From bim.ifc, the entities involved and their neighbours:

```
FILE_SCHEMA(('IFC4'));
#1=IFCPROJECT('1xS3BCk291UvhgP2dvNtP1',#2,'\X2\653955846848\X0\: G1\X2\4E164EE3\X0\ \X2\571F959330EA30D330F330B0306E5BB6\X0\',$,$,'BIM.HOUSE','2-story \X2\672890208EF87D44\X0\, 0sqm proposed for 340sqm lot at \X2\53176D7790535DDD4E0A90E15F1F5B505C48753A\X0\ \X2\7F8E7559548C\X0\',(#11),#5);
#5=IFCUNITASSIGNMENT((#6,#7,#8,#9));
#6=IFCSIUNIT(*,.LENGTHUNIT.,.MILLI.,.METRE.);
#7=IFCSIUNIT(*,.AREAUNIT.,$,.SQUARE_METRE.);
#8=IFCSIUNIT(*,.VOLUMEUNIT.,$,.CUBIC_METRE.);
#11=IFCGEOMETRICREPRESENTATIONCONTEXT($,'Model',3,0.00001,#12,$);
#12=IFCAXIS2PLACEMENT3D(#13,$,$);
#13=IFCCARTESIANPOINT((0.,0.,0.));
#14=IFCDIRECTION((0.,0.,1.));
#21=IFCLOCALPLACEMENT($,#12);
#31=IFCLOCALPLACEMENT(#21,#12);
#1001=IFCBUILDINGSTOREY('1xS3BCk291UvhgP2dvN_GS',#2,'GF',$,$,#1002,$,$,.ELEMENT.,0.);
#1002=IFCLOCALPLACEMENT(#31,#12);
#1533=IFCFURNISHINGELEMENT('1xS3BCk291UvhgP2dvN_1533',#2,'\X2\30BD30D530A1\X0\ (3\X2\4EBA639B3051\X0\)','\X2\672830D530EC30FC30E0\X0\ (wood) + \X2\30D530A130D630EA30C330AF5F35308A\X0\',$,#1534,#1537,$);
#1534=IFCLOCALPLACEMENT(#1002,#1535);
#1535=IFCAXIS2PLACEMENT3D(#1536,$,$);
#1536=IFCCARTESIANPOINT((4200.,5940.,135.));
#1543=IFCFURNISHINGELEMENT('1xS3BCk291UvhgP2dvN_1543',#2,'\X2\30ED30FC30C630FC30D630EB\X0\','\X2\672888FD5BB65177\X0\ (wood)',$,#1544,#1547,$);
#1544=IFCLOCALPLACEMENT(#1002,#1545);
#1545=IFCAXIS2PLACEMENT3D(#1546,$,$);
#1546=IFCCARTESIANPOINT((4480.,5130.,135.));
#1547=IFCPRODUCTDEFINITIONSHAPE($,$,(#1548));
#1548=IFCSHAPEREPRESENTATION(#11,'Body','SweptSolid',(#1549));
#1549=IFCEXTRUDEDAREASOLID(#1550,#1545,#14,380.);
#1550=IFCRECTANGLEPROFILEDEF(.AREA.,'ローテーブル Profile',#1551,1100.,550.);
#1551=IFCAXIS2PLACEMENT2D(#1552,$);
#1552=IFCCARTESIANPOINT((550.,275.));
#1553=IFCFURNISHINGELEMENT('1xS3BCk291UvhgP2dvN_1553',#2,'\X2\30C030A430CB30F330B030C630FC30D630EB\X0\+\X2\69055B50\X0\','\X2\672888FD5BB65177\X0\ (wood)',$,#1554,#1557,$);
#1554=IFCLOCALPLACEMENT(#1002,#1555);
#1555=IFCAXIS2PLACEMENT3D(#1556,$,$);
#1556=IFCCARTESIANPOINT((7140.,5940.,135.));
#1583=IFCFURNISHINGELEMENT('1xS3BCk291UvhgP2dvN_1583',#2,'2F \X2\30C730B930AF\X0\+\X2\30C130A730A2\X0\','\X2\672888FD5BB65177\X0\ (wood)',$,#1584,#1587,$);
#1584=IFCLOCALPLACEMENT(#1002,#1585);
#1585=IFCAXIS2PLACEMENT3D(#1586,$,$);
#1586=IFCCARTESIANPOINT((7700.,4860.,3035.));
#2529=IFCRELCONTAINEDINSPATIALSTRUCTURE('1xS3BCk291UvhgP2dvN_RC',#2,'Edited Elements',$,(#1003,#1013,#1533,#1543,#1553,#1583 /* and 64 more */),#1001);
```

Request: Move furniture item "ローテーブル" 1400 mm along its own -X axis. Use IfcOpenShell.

```python
import ifcopenshell
import ifcopenshell.api.geometry
import ifcopenshell.util.placement

model = ifcopenshell.open("bim.ifc")

item = model.by_guid("1xS3BCk291UvhgP2dvN_1543")
matrix = ifcopenshell.util.placement.get_local_placement(item.ObjectPlacement)
matrix[:3, 3] -= matrix[:3, 0] * 1400.0
ifcopenshell.api.geometry.edit_object_placement(model, product=item, matrix=matrix, is_si=False)

print(ifcopenshell.util.placement.get_local_placement(item.ObjectPlacement).round(3) + 0.0)

model.write("bim_v2.ifc")
```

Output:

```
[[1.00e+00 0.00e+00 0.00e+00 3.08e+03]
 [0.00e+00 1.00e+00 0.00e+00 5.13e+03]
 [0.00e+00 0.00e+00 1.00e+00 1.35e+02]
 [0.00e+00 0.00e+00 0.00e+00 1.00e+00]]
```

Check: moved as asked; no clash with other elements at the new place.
